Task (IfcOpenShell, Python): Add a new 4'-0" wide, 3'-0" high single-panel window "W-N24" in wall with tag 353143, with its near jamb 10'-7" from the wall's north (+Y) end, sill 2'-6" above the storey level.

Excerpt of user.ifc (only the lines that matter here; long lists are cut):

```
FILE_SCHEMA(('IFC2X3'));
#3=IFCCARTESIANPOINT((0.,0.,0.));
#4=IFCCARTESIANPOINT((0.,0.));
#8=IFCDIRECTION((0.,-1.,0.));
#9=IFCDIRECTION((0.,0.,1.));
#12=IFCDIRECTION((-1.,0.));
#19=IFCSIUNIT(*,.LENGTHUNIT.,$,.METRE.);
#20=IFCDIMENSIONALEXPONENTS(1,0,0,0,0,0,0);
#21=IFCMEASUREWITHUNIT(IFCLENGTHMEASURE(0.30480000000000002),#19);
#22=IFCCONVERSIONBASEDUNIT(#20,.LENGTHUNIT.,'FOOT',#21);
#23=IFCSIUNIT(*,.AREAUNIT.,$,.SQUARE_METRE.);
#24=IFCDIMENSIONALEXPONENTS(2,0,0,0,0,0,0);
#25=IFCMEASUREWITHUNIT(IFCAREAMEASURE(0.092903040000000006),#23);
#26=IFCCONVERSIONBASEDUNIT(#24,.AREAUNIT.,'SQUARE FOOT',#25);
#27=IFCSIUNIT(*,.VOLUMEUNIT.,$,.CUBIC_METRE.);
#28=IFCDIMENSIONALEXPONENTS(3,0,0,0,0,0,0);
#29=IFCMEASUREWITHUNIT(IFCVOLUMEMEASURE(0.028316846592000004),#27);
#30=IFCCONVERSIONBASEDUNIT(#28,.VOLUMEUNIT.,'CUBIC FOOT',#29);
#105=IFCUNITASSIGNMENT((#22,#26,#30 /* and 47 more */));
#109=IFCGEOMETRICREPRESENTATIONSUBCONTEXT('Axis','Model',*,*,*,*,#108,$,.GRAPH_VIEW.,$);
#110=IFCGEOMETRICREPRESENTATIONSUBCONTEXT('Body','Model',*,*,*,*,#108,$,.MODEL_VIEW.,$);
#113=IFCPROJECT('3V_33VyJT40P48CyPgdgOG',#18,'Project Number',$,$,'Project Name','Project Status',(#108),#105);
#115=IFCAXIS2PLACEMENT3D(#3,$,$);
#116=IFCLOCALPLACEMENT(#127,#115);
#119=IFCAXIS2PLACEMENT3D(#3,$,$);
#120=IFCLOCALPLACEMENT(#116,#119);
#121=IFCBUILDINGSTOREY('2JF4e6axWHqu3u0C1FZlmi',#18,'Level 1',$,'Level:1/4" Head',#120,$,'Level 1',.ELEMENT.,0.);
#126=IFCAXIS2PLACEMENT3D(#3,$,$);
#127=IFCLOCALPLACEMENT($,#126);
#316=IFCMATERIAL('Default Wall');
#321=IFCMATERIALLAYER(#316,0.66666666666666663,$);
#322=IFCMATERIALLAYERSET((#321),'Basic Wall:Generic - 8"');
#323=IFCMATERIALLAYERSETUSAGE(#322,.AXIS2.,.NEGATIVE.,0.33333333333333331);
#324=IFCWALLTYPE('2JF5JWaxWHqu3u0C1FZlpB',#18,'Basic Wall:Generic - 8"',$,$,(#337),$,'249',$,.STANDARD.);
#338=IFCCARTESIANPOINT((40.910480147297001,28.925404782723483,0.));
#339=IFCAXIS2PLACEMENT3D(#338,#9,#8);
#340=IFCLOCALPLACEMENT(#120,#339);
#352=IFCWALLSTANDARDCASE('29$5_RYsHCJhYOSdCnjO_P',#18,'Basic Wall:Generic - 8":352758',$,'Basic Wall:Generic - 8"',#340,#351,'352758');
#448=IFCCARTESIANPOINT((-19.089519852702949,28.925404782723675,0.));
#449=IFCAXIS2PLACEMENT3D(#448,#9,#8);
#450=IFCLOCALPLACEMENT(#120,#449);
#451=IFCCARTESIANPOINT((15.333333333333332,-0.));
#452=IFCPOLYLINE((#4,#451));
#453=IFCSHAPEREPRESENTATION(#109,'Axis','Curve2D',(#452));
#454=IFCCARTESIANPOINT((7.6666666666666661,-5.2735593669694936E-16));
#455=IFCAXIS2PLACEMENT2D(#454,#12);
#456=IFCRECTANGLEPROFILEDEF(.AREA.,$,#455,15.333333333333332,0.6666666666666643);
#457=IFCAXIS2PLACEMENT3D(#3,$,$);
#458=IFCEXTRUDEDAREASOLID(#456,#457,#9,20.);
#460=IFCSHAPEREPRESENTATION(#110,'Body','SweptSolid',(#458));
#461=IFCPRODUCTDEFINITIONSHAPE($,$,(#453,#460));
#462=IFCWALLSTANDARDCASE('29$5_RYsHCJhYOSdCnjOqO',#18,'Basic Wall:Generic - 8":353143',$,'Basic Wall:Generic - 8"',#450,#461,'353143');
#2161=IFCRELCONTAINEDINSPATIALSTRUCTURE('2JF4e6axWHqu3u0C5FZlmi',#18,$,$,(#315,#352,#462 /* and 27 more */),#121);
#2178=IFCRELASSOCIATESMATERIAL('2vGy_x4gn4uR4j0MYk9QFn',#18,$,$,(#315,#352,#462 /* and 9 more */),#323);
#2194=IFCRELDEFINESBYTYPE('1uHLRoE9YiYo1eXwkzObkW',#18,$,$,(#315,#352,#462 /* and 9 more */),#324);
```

```python
import numpy as np
import ifcopenshell
import ifcopenshell.api.feature
import ifcopenshell.api.geometry
import ifcopenshell.api.root
import ifcopenshell.api.spatial
import ifcopenshell.api.type
import ifcopenshell.geom
import ifcopenshell.util.element
import ifcopenshell.util.placement
import ifcopenshell.util.representation
import ifcopenshell.util.shape
import ifcopenshell.util.unit

model = ifcopenshell.open("user.ifc")
unit_scale = ifcopenshell.util.unit.calculate_unit_scale(model)
settings = ifcopenshell.geom.settings()


def volume(element):
    """Net volume in cubic metres, openings subtracted."""
    shape = ifcopenshell.geom.create_shape(settings, element)
    return ifcopenshell.util.shape.get_volume(shape.geometry)


wall = model.by_guid("29$5_RYsHCJhYOSdCnjOqO")
storey = ifcopenshell.util.element.get_container(wall, ifc_class="IfcBuildingStorey")
context = ifcopenshell.util.representation.get_context(model, "Model", "Body", "MODEL_VIEW")
before = volume(wall)

width, height, from_end, sill = 1.2192, 0.9144, 3.2258, 0.762  # metres

# The wall runs along its own X axis, and the end named is its -X end.
wall_shape = ifcopenshell.geom.create_shape(settings, wall)
x, y, z = ifcopenshell.util.shape.get_vertices(wall_shape.geometry).T
start = x.min() + from_end
face, thickness = float(y.min()), float(y.max() - y.min())
wall_matrix = ifcopenshell.util.placement.get_local_placement(wall.ObjectPlacement)
level = ifcopenshell.util.placement.get_local_placement(storey.ObjectPlacement)[2, 3]


def in_wall(x, y):
    """Placement at x, y metres in the wall's axes, at sill height."""
    matrix = wall_matrix.copy()
    matrix[:, 3] = wall_matrix @ np.array([x / unit_scale, y / unit_scale, 0.0, 1.0])
    matrix[2, 3] = level + sill / unit_scale
    return matrix


# Opening: a box that overshoots both wall faces by 50 mm.
opening = ifcopenshell.api.root.create_entity(model, ifc_class="IfcOpeningElement")
box = ifcopenshell.api.geometry.add_wall_representation(
    model, context=context, length=width, height=height, thickness=thickness + 0.1
)
ifcopenshell.api.geometry.assign_representation(model, product=opening, representation=box)
ifcopenshell.api.geometry.edit_object_placement(model, product=opening, matrix=in_wall(start, face - 0.05), is_si=False)
ifcopenshell.api.feature.add_feature(model, feature=opening, element=wall)

window = ifcopenshell.api.root.create_entity(model, ifc_class="IfcWindow", name="W-N24")
window.OverallWidth, window.OverallHeight = width / unit_scale, height / unit_scale
body = ifcopenshell.api.geometry.add_window_representation(
    model,
    context=context,
    overall_width=window.OverallWidth,
    overall_height=window.OverallHeight,
    partition_type="SINGLE_PANEL",
)
ifcopenshell.api.geometry.assign_representation(model, product=window, representation=body)
ifcopenshell.api.spatial.assign_container(model, products=[window], relating_structure=storey)
fills = ifcopenshell.api.feature.add_filling(model, opening=opening, element=window)
fills.OwnerHistory = window.OwnerHistory  # required in IFC2X3

# IFC2X3 keeps the operation on the window style.
style = ifcopenshell.api.root.create_entity(model, ifc_class="IfcWindowStyle", name="W-N24")
style.OperationType, style.ConstructionType = "SINGLE_PANEL", "NOTDEFINED"
style.ParameterTakesPrecedence = style.Sizeable = False
ifcopenshell.api.type.assign_type(model, related_objects=[window], relating_type=style)

# Centre the window in the wall's thickness.
ifcopenshell.api.geometry.edit_object_placement(model, product=window, matrix=in_wall(start, face), is_si=False)
window_shape = ifcopenshell.geom.create_shape(settings, window)
depth = ifcopenshell.util.shape.get_vertices(window_shape.geometry)[:, 1]
offset = face + thickness / 2 - (depth.min() + depth.max()) / 2
ifcopenshell.api.geometry.edit_object_placement(model, product=window, matrix=in_wall(start, offset), is_si=False)

after = volume(wall)

print(f"wall volume {before:.3f} -> {after:.3f} m3")

model.write("user_v2.ifc")
```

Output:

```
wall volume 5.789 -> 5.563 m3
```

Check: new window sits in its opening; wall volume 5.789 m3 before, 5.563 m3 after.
